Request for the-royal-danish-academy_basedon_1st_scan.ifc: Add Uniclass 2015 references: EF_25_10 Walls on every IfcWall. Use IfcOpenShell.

First a look at what the model holds.

```python
import ifcopenshell

model = ifcopenshell.open("the-royal-danish-academy_basedon_1st_scan.ifc")
print(model.schema)
print("classifications:", [c.Name for c in model.by_type("IfcClassification")])
for ifc_class in ("IfcDoor", "IfcRoof", "IfcStair", "IfcWall", "IfcWindow"):
    print(ifc_class, len(model.by_type(ifc_class)))
```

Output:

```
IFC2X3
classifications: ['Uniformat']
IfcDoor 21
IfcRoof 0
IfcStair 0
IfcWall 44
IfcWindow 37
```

```python
import ifcopenshell
import ifcopenshell.api.classification

model = ifcopenshell.open("the-royal-danish-academy_basedon_1st_scan.ifc")

# IFC2X3 requires Source and Edition and has no link from the project to the system.
system = model.create_entity("IfcClassification", Source="NBS", Edition="2015", Name="Uniclass 2015")

codes = {
    "IfcWall": ("EF_25_10", "Walls"),
}
for ifc_class, (code, name) in codes.items():
    products = model.by_type(ifc_class)
    ifcopenshell.api.classification.add_reference(
        model, products=products, classification=system, identification=code, name=name
    )
    print(code, len(products))

model.write("the-royal-danish-academy_basedon_1st_scan_v2.ifc")
```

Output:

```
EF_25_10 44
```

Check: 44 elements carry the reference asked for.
